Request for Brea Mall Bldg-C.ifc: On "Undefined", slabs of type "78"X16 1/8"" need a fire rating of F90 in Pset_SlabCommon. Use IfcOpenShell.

First a look at what the model holds.

```python
import ifcopenshell
import ifcopenshell.util.element

model = ifcopenshell.open("Brea Mall Bldg-C.ifc")
print(model.schema)
storey = next(s for s in model.by_type("IfcBuildingStorey") if s.Name == "Undefined")
slabs = [e for e in ifcopenshell.util.element.get_decomposition(storey) if e.is_a("IfcSlab")]
seen = {}
for e in slabs:
    element_type = ifcopenshell.util.element.get_type(e)
    key = (element_type.Name if element_type != e and element_type else None, ifcopenshell.util.element.get_pset(e, "Pset_SlabCommon", "FireRating"))
    seen[key] = seen.get(key, 0) + 1
for (name, value), count in sorted(seen.items(), key=str):
    print(count, "x", name, "|", value)
```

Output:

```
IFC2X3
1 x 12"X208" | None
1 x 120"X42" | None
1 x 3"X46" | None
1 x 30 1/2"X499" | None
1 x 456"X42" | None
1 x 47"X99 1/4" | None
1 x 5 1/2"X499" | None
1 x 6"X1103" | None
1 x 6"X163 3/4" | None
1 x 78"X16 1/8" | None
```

```python
import ifcopenshell
import ifcopenshell.api.pset
import ifcopenshell.util.element

model = ifcopenshell.open("Brea Mall Bldg-C.ifc")

storey = next(s for s in model.by_type("IfcBuildingStorey") if s.Name == "Undefined")
slabs = [e for e in ifcopenshell.util.element.get_decomposition(storey) if e.is_a("IfcSlab")]

count = 0
for e in slabs:
    element_type = ifcopenshell.util.element.get_type(e)
    if element_type in (None, e) or element_type.Name != '78"X16 1/8"':
        continue
    # add_pset returns the element's existing set when there is one.
    pset = ifcopenshell.api.pset.add_pset(model, product=e, name="Pset_SlabCommon")
    ifcopenshell.api.pset.edit_pset(model, pset=pset, properties={"FireRating": "F90"})
    count += 1

print(count, "slabs updated")

model.write("Brea Mall Bldg-C_edited.ifc")
```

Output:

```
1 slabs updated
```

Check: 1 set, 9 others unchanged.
